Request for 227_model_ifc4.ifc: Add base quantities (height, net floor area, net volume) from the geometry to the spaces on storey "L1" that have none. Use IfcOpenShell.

First a look at what the model holds.

```python
import ifcopenshell
import ifcopenshell.util.element
import ifcopenshell.util.unit

model = ifcopenshell.open("227_model_ifc4.ifc")
print(model.schema)
for unit_type in ("LENGTHUNIT", "AREAUNIT", "VOLUMEUNIT"):
    print(unit_type, ifcopenshell.util.unit.calculate_unit_scale(model, unit_type))
storey = next(s for s in model.by_type("IfcBuildingStorey") if s.Name == "L1")
spaces = [e for e in ifcopenshell.util.element.get_decomposition(storey) if e.is_a("IfcSpace")]
for e in sorted(spaces, key=lambda e: e.id()):
    print(e.id(), e.is_a(), e.Name, list(ifcopenshell.util.element.get_psets(e, qtos_only=True)), sep=" | ")
```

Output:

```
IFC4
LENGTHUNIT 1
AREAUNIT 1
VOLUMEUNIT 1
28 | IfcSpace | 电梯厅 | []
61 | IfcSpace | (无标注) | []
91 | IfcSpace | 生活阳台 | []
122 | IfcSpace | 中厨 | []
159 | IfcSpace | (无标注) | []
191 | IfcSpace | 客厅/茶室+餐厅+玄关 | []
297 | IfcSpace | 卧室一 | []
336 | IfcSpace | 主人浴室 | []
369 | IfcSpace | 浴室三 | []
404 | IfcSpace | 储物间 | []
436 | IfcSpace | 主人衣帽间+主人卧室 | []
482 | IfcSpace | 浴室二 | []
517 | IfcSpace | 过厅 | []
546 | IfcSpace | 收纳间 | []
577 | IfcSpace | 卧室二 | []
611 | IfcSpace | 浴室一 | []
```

```python
import ifcopenshell
import ifcopenshell.api.pset
import ifcopenshell.geom
import ifcopenshell.util.element
import ifcopenshell.util.shape
import ifcopenshell.util.unit

model = ifcopenshell.open("227_model_ifc4.ifc")
unit_scale = ifcopenshell.util.unit.calculate_unit_scale(model)
area_scale = ifcopenshell.util.unit.calculate_unit_scale(model, "AREAUNIT")
volume_scale = ifcopenshell.util.unit.calculate_unit_scale(model, "VOLUMEUNIT")
settings = ifcopenshell.geom.settings()

storey = next(s for s in model.by_type("IfcBuildingStorey") if s.Name == "L1")
spaces = [e for e in ifcopenshell.util.element.get_decomposition(storey) if e.is_a("IfcSpace")]

for e in sorted(spaces, key=lambda e: e.id()):
    if ifcopenshell.util.element.get_psets(e, qtos_only=True, should_inherit=False):
        continue
    # Geometry comes back in metres, in the element's own axes.
    shape = ifcopenshell.geom.create_shape(settings, e)
    values = {
        "Height": ifcopenshell.util.shape.get_z(shape.geometry) / unit_scale,
        "NetFloorArea": ifcopenshell.util.shape.get_footprint_area(shape.geometry) / area_scale,
        "NetVolume": ifcopenshell.util.shape.get_volume(shape.geometry) / volume_scale,
    }
    qto = ifcopenshell.api.pset.add_qto(model, product=e, name="Qto_SpaceBaseQuantities")
    ifcopenshell.api.pset.edit_qto(model, qto=qto, properties=values)
    print(e.id(), {k: round(v, 3) for k, v in values.items()})

model.write("227_model_ifc4-out.ifc")
```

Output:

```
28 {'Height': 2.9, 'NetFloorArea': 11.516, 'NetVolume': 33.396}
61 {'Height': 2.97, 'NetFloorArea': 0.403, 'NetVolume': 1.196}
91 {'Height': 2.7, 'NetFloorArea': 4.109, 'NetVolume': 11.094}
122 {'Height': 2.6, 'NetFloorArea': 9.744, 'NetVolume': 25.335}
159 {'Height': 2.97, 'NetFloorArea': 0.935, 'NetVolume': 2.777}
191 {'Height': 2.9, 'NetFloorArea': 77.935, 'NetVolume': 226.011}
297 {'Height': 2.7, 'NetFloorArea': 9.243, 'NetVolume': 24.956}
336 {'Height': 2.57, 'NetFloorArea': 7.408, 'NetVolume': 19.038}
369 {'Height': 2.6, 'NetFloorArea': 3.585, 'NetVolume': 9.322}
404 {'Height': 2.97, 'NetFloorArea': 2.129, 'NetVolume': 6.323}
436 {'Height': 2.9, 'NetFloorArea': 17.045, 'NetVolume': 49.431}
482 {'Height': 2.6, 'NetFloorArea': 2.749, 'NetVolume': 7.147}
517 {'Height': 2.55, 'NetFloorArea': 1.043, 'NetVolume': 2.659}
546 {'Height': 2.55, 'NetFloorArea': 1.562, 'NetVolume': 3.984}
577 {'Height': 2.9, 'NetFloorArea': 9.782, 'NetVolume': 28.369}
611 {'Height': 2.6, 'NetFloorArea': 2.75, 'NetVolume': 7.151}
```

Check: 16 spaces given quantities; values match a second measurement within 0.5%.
